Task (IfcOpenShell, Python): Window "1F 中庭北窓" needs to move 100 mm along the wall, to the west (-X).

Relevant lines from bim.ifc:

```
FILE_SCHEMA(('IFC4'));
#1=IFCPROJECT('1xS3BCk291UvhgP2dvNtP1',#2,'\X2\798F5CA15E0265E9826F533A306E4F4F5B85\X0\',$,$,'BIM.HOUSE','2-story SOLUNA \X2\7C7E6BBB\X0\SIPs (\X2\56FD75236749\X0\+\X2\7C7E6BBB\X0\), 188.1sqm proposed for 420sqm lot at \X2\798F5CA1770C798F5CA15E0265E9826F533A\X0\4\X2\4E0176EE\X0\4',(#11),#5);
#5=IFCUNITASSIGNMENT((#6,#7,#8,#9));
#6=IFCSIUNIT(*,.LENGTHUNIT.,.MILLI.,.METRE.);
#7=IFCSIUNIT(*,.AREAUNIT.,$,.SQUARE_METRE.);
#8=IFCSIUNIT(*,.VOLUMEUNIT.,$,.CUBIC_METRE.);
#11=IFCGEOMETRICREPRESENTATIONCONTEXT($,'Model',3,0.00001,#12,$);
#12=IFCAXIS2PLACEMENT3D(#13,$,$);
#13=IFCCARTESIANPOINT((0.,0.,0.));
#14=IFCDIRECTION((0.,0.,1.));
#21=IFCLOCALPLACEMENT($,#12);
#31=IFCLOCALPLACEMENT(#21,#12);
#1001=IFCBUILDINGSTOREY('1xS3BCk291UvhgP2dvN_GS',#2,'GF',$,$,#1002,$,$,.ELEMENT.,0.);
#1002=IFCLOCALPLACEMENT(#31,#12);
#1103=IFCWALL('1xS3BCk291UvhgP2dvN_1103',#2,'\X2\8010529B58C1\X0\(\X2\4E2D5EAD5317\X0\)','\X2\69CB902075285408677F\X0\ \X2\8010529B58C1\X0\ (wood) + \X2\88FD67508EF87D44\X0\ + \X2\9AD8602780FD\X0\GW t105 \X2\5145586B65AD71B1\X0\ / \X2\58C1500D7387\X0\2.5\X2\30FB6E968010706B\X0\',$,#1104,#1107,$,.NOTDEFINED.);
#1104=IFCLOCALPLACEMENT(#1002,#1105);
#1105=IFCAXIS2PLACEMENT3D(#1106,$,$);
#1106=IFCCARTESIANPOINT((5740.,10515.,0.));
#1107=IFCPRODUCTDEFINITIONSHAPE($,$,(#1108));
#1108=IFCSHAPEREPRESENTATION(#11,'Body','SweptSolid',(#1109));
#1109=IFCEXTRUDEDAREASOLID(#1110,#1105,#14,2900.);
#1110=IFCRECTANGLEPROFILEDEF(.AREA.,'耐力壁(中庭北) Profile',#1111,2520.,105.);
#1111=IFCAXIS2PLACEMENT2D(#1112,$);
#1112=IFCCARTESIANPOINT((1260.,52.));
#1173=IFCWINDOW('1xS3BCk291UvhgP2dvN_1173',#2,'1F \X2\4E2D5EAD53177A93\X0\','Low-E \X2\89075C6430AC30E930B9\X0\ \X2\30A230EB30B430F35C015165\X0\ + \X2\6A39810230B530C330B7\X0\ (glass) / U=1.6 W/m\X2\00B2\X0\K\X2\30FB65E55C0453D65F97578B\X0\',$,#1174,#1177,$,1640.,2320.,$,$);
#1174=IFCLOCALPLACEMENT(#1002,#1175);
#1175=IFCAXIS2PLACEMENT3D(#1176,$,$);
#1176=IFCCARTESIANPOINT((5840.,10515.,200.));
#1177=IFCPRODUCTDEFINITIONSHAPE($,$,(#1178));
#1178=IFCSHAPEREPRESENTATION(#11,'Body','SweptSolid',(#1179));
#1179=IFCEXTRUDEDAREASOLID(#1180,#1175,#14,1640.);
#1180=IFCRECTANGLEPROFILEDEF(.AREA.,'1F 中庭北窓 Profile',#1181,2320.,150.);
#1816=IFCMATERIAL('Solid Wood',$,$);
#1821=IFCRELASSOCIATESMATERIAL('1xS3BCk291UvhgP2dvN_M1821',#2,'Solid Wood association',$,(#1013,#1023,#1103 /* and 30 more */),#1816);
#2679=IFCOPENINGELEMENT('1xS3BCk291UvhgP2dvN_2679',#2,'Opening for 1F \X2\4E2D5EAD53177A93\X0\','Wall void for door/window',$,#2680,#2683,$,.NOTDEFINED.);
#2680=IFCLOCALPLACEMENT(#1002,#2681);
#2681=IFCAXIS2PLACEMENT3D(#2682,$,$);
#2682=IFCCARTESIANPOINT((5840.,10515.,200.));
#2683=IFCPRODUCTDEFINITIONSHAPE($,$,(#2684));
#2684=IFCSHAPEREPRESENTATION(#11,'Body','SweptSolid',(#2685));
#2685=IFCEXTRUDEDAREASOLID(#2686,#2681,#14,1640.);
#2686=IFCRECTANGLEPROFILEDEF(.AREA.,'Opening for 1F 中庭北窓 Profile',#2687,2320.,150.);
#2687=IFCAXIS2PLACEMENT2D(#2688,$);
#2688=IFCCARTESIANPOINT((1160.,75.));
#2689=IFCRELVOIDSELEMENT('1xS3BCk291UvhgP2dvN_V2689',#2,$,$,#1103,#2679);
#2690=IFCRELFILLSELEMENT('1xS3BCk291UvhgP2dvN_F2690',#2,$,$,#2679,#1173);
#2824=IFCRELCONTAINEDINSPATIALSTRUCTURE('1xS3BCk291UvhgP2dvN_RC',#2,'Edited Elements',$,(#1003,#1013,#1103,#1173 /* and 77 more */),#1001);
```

```python
import ifcopenshell
import ifcopenshell.api.geometry
import ifcopenshell.util.placement

model = ifcopenshell.open("bim.ifc")

window = model.by_id(1173)
opening = window.FillsVoids[0].RelatingOpeningElement
wall = opening.VoidsElements[0].RelatingBuildingElement

wall_matrix = ifcopenshell.util.placement.get_local_placement(wall.ObjectPlacement)
shift = wall_matrix[:3, 0] * -100.0
before = ifcopenshell.util.placement.get_local_placement(window.ObjectPlacement)[:3, 3].copy()

# The window is not placed relative to its opening, so move both.
for product in (opening, window):
    matrix = ifcopenshell.util.placement.get_local_placement(product.ObjectPlacement)
    matrix[:3, 3] += shift
    ifcopenshell.api.geometry.edit_object_placement(model, product=product, matrix=matrix, is_si=False)

after = ifcopenshell.util.placement.get_local_placement(window.ObjectPlacement)[:3, 3]
print("window moved by", (after - before).round(3) + 0.0)

model.write("bim-out.ifc")
```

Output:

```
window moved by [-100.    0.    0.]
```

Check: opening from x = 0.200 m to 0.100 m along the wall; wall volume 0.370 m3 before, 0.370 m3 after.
